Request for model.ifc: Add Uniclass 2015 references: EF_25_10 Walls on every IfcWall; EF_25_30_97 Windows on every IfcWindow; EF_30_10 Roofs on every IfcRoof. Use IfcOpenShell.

First a look at what the model holds.

```python
import ifcopenshell

model = ifcopenshell.open("model.ifc")
print(model.schema)
print("classifications:", [c.Name for c in model.by_type("IfcClassification")])
for ifc_class in ("IfcDoor", "IfcRoof", "IfcStair", "IfcWall", "IfcWindow"):
    print(ifc_class, len(model.by_type(ifc_class)))
```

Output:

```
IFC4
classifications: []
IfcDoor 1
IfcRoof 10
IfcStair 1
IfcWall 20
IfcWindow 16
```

```python
import ifcopenshell
import ifcopenshell.api.classification

model = ifcopenshell.open("model.ifc")

system = ifcopenshell.api.classification.add_classification(model, classification="Uniclass 2015")

codes = {
    "IfcWall": ("EF_25_10", "Walls"),
    "IfcWindow": ("EF_25_30_97", "Windows"),
    "IfcRoof": ("EF_30_10", "Roofs"),
}
for ifc_class, (code, name) in codes.items():
    products = model.by_type(ifc_class)
    ifcopenshell.api.classification.add_reference(
        model, products=products, classification=system, identification=code, name=name
    )
    print(code, len(products))

model.write("model_updated.ifc")
```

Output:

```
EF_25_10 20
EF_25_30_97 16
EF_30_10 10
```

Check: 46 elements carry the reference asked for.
